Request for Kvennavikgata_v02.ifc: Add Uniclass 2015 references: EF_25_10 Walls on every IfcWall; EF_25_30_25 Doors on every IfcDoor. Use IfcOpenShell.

First a look at what the model holds.

```python
import ifcopenshell

model = ifcopenshell.open("Kvennavikgata_v02.ifc")
print(model.schema)
print("classifications:", [c.Name for c in model.by_type("IfcClassification")])
for ifc_class in ("IfcDoor", "IfcRoof", "IfcStair", "IfcWall", "IfcWindow"):
    print(ifc_class, len(model.by_type(ifc_class)))
```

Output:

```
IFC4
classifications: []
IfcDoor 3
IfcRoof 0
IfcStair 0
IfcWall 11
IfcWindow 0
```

```python
import ifcopenshell
import ifcopenshell.api.classification

model = ifcopenshell.open("Kvennavikgata_v02.ifc")

system = ifcopenshell.api.classification.add_classification(model, classification="Uniclass 2015")

codes = {
    "IfcWall": ("EF_25_10", "Walls"),
    "IfcDoor": ("EF_25_30_25", "Doors"),
}
for ifc_class, (code, name) in codes.items():
    products = model.by_type(ifc_class)
    ifcopenshell.api.classification.add_reference(
        model, products=products, classification=system, identification=code, name=name
    )
    print(code, len(products))

model.write("Kvennavikgata_v02_updated.ifc")
```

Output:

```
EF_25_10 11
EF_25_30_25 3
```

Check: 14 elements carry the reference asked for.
